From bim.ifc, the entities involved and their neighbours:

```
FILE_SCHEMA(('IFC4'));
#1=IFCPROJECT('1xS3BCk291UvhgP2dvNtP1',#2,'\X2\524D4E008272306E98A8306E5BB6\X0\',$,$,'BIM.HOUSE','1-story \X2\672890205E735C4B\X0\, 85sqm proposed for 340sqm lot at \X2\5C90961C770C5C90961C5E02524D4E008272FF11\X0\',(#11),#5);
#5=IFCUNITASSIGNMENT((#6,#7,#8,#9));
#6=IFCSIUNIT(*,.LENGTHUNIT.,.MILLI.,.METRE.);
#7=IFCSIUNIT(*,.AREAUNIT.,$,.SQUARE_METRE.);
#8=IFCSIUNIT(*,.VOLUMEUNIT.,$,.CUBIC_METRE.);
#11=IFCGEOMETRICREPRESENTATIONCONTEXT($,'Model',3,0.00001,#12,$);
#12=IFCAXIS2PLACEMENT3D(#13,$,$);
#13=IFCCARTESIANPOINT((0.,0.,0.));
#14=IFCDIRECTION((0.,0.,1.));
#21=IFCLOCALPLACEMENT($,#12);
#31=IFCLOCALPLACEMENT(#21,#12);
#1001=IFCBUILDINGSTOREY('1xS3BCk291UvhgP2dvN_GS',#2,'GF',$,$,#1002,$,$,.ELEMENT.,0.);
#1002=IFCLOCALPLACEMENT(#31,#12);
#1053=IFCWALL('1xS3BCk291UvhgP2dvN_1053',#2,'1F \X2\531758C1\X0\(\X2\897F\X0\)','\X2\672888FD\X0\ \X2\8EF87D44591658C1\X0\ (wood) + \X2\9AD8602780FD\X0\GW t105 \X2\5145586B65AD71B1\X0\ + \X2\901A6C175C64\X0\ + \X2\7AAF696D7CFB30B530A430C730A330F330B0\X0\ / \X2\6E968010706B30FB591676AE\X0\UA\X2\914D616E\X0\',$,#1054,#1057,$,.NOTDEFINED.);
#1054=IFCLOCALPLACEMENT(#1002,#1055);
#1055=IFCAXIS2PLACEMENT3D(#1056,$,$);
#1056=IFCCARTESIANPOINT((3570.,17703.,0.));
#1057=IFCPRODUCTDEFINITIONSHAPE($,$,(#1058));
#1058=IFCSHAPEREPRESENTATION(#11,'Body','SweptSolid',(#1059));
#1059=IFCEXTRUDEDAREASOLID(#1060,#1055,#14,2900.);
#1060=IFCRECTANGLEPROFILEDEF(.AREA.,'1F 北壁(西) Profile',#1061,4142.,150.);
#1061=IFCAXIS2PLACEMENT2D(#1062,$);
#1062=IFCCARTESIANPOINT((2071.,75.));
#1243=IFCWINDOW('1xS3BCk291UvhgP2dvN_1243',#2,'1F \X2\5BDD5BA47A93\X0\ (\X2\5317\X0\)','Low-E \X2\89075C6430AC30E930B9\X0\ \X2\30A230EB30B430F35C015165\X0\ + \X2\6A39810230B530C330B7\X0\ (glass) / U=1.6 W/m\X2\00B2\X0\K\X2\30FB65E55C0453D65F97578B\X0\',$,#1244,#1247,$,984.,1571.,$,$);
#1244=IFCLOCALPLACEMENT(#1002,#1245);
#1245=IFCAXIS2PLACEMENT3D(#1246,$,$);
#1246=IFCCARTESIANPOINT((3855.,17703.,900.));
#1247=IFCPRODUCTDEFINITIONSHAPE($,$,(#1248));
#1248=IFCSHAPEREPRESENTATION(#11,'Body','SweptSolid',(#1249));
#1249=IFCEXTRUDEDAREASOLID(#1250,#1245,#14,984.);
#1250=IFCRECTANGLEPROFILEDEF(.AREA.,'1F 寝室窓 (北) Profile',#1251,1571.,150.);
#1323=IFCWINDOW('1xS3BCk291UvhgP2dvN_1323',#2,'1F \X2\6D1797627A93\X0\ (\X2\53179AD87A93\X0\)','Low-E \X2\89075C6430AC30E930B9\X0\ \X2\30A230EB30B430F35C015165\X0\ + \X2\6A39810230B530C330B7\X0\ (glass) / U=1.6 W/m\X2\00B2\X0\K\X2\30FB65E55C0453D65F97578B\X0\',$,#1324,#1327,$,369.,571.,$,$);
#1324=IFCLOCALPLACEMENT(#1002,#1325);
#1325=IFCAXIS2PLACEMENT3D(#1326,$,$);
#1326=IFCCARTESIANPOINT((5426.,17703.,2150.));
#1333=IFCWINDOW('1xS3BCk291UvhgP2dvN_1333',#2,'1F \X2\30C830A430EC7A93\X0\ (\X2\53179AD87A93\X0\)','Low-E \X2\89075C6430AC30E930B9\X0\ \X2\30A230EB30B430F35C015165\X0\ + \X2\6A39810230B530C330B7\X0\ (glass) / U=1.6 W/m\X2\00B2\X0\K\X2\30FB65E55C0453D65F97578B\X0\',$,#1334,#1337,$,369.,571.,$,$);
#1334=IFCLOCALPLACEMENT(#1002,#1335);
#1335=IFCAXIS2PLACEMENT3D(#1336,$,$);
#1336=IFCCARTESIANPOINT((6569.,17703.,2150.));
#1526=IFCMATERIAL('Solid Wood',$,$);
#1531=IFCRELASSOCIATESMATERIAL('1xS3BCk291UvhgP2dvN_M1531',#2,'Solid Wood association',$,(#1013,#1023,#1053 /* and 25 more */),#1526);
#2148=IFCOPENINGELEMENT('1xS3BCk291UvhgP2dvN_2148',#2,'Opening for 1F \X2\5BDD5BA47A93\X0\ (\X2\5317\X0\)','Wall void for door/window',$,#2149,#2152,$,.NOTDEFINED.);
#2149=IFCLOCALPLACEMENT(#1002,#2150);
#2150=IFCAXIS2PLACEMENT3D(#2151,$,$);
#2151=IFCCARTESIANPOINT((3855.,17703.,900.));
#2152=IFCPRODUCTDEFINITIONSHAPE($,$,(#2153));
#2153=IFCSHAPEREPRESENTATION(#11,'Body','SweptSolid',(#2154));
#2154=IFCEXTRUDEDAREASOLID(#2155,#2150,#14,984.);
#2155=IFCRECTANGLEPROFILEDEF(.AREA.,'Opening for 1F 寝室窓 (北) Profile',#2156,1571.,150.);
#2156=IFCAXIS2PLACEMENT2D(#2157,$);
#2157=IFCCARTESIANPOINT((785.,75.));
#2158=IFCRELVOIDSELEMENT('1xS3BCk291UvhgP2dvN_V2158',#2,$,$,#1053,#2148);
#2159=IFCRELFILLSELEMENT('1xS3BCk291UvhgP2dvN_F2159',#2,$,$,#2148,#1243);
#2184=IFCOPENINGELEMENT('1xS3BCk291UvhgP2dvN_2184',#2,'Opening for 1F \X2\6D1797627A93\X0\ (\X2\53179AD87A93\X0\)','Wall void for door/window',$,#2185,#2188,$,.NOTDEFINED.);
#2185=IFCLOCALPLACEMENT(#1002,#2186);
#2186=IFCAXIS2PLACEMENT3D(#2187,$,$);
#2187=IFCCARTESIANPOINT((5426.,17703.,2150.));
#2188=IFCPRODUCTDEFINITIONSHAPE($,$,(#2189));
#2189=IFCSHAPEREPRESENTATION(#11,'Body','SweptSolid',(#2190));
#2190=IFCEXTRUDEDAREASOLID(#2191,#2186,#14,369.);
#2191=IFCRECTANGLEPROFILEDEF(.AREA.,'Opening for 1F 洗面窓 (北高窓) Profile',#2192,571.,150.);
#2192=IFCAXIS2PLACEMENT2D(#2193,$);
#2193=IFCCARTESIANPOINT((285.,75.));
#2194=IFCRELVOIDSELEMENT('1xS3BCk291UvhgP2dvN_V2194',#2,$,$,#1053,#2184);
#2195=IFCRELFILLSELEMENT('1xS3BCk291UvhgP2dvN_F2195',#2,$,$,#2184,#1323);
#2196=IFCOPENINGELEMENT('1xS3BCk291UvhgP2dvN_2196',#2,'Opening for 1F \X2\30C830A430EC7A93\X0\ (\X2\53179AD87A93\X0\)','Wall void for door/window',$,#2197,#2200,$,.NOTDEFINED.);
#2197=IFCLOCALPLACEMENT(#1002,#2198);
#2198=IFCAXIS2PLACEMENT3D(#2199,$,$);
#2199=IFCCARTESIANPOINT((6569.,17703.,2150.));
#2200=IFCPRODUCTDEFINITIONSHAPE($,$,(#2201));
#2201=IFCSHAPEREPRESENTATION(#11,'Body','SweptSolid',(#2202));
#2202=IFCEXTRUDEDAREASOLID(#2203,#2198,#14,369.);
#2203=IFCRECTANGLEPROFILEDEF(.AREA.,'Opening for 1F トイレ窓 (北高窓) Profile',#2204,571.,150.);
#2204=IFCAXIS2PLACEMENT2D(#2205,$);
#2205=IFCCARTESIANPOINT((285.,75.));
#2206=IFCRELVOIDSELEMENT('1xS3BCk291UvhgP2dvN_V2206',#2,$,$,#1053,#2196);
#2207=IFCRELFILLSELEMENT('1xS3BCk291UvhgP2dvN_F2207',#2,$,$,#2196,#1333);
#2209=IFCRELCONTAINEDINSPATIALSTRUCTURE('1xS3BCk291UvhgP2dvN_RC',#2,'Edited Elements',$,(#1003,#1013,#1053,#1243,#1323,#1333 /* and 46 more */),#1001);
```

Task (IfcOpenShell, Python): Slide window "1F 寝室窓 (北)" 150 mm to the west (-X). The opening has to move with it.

```python
import ifcopenshell
import ifcopenshell.api.geometry
import ifcopenshell.util.placement
import ifcopenshell.util.unit

model = ifcopenshell.open("bim.ifc")
unit_scale = ifcopenshell.util.unit.calculate_unit_scale(model)

window = model.by_guid("1xS3BCk291UvhgP2dvN_1243")
opening = window.FillsVoids[0].RelatingOpeningElement
wall = opening.VoidsElements[0].RelatingBuildingElement

wall_matrix = ifcopenshell.util.placement.get_local_placement(wall.ObjectPlacement)
shift = wall_matrix[:3, 0] * -0.15 / unit_scale
before = ifcopenshell.util.placement.get_local_placement(window.ObjectPlacement)[:3, 3].copy()

# The window is not placed relative to its opening, so move both.
for product in (opening, window):
    matrix = ifcopenshell.util.placement.get_local_placement(product.ObjectPlacement)
    matrix[:3, 3] += shift
    ifcopenshell.api.geometry.edit_object_placement(model, product=product, matrix=matrix, is_si=False)

after = ifcopenshell.util.placement.get_local_placement(window.ObjectPlacement)[:3, 3]
print("window moved by", (after - before).round(3) + 0.0)

model.write("bim_v2.ifc")
```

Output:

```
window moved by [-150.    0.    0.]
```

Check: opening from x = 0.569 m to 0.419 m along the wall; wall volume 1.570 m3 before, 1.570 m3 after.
